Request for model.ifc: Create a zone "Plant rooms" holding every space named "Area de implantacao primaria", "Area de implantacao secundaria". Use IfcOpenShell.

First a look at what the model holds.

```python
import ifcopenshell

model = ifcopenshell.open("model.ifc")
print(model.schema)
seen = {}
for space in model.by_type("IfcSpace"):
    seen[space.LongName] = seen.get(space.LongName, 0) + 1
for name, count in sorted(seen.items(), key=str):
    print(count, "x", name)
print("zones:", [z.Name for z in model.by_type("IfcZone")][:20])
```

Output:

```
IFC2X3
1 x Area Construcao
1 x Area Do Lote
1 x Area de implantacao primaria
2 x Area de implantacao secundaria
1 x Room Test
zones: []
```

```python
import ifcopenshell
import ifcopenshell.api.group
import ifcopenshell.api.root

model = ifcopenshell.open("model.ifc")

names = {"Area de implantacao primaria", "Area de implantacao secundaria"}
spaces = [s for s in model.by_type("IfcSpace") if s.LongName in names]

zone = ifcopenshell.api.root.create_entity(model, ifc_class="IfcZone", name="Plant rooms")
ifcopenshell.api.group.assign_group(model, products=spaces, group=zone)
print(len(spaces), "spaces in", zone.Name)

model.write("model_edited.ifc")
```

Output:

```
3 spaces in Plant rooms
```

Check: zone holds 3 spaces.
